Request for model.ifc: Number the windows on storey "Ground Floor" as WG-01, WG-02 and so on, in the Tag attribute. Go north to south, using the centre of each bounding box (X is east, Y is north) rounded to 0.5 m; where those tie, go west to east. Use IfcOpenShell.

First a look at what the model holds.

```python
import ifcopenshell
import ifcopenshell.util.element
import ifcopenshell.util.placement

model = ifcopenshell.open("model.ifc")
print(model.schema)
storey = next(s for s in model.by_type("IfcBuildingStorey") if s.Name == "Ground Floor")
windows = [e for e in ifcopenshell.util.element.get_decomposition(storey) if e.is_a("IfcWindow")]
for e in sorted(windows, key=lambda e: e.id()):
    origin = ifcopenshell.util.placement.get_local_placement(e.ObjectPlacement)[:3, 3]
    print(e.id(), e.Tag, e.Name, origin.round(2) + 0.0, sep=" | ")
```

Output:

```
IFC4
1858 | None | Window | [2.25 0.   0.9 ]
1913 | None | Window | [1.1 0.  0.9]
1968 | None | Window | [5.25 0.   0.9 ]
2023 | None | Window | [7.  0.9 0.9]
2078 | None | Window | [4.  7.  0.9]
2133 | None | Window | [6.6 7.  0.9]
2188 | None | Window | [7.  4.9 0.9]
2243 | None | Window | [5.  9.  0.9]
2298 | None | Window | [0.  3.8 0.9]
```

```python
import ifcopenshell
import ifcopenshell.geom
import ifcopenshell.util.element
import ifcopenshell.util.shape

model = ifcopenshell.open("model.ifc")
settings = ifcopenshell.geom.settings()
settings.set("use-world-coords", True)


def centre(element):
    shape = ifcopenshell.geom.create_shape(settings, element)
    return ifcopenshell.util.shape.get_bbox_centroid(shape.geometry)


storey = next(s for s in model.by_type("IfcBuildingStorey") if s.Name == "Ground Floor")
windows = [e for e in ifcopenshell.util.element.get_decomposition(storey) if e.is_a("IfcWindow")]

# Insertion points can sit at a corner or the storey origin, so sort by the geometry (in metres).
centres = {e: centre(e) for e in windows}
windows.sort(key=lambda e: (-round(centres[e][1] / 0.5), centres[e][0]))

for i, e in enumerate(windows, start=1):
    number = f"WG-{i:02d}"
    e.Tag = number
    print(e.id(), number)

model.write("model_rev.ifc")
```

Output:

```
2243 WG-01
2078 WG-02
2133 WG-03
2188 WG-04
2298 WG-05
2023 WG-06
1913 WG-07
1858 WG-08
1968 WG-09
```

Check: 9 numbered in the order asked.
